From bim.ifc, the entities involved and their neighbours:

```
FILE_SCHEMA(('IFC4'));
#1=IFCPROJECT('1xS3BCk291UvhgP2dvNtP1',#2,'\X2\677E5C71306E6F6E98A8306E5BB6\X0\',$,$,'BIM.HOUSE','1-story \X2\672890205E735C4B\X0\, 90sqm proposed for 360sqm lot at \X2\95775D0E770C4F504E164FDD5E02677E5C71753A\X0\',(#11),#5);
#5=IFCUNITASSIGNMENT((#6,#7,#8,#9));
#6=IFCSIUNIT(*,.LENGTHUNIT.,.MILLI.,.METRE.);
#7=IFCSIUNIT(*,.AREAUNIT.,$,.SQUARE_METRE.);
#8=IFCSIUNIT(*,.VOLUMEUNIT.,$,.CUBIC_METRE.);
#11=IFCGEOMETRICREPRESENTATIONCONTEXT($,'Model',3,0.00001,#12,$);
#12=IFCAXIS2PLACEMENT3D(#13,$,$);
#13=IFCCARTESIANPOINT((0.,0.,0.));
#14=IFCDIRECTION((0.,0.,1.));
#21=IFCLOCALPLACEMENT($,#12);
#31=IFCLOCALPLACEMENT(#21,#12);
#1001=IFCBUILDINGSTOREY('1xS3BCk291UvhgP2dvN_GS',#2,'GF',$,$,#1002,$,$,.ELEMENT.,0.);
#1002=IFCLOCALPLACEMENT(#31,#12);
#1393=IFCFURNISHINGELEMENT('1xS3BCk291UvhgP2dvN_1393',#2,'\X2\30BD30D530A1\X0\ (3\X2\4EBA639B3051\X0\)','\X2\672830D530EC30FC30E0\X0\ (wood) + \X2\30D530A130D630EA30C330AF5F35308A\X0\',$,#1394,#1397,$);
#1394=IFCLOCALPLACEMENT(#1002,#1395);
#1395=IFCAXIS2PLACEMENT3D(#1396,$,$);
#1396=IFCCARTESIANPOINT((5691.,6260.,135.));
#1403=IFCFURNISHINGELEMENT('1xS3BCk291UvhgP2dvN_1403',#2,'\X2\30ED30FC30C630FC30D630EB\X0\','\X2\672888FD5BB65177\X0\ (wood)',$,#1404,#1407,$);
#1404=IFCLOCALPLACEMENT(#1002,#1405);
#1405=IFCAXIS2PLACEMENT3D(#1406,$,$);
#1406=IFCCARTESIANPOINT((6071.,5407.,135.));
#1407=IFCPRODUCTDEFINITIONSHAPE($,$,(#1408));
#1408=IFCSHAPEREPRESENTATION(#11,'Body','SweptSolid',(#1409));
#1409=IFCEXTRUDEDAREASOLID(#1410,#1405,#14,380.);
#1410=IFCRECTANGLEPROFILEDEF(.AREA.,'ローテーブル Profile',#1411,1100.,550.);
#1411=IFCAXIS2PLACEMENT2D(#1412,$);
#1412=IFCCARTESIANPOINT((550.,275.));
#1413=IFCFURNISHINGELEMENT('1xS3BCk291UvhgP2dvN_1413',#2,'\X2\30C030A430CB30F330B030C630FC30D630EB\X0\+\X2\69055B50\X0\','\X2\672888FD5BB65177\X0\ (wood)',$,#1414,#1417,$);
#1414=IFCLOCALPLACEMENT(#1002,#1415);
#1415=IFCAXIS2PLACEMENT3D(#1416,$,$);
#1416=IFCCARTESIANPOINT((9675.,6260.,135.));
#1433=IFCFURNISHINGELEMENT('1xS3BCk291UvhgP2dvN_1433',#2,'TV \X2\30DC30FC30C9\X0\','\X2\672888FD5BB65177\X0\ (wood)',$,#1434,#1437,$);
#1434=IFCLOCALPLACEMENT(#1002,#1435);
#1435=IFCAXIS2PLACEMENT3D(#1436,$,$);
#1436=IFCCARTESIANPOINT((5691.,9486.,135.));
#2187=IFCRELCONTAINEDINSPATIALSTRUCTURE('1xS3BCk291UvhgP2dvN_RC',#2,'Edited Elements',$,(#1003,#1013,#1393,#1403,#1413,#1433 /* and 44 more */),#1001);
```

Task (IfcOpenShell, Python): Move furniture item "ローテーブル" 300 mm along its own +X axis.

```python
import ifcopenshell
import ifcopenshell.api.geometry
import ifcopenshell.util.placement

model = ifcopenshell.open("bim.ifc")

item = model.by_id(1403)
matrix = ifcopenshell.util.placement.get_local_placement(item.ObjectPlacement)
matrix[:3, 3] += matrix[:3, 0] * 300.0
ifcopenshell.api.geometry.edit_object_placement(model, product=item, matrix=matrix, is_si=False)

print(ifcopenshell.util.placement.get_local_placement(item.ObjectPlacement).round(3) + 0.0)

model.write("bim_updated.ifc")
```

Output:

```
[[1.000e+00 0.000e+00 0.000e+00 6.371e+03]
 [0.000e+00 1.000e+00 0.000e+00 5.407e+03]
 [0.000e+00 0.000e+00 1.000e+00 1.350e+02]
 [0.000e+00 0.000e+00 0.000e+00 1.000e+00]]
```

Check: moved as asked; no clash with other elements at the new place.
